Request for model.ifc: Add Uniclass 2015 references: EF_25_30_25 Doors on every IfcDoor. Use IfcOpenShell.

First a look at what the model holds.

```python
import ifcopenshell

model = ifcopenshell.open("model.ifc")
print(model.schema)
print("classifications:", [c.Name for c in model.by_type("IfcClassification")])
for ifc_class in ("IfcDoor", "IfcRoof", "IfcStair", "IfcWall", "IfcWindow"):
    print(ifc_class, len(model.by_type(ifc_class)))
```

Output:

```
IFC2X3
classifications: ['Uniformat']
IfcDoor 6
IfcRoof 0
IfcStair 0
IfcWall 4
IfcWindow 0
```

```python
import ifcopenshell
import ifcopenshell.api.classification

model = ifcopenshell.open("model.ifc")

# IFC2X3 requires Source and Edition and has no link from the project to the system.
system = model.create_entity("IfcClassification", Source="NBS", Edition="2015", Name="Uniclass 2015")

codes = {
    "IfcDoor": ("EF_25_30_25", "Doors"),
}
for ifc_class, (code, name) in codes.items():
    products = model.by_type(ifc_class)
    ifcopenshell.api.classification.add_reference(
        model, products=products, classification=system, identification=code, name=name
    )
    print(code, len(products))

model.write("model_v2.ifc")
```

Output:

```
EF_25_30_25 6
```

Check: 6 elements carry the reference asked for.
